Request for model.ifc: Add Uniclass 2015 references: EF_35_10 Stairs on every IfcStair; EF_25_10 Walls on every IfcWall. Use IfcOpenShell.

First a look at what the model holds.

```python
import ifcopenshell

model = ifcopenshell.open("model.ifc")
print(model.schema)
print("classifications:", [c.Name for c in model.by_type("IfcClassification")])
for ifc_class in ("IfcDoor", "IfcRoof", "IfcStair", "IfcWall", "IfcWindow"):
    print(ifc_class, len(model.by_type(ifc_class)))
```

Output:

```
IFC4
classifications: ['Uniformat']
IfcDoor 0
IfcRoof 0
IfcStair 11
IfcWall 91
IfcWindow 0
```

```python
import ifcopenshell
import ifcopenshell.api.classification

model = ifcopenshell.open("model.ifc")

system = ifcopenshell.api.classification.add_classification(model, classification="Uniclass 2015")

codes = {
    "IfcStair": ("EF_35_10", "Stairs"),
    "IfcWall": ("EF_25_10", "Walls"),
}
for ifc_class, (code, name) in codes.items():
    products = model.by_type(ifc_class)
    ifcopenshell.api.classification.add_reference(
        model, products=products, classification=system, identification=code, name=name
    )
    print(code, len(products))

model.write("model_rev.ifc")
```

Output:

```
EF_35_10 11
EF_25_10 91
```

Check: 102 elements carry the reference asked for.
